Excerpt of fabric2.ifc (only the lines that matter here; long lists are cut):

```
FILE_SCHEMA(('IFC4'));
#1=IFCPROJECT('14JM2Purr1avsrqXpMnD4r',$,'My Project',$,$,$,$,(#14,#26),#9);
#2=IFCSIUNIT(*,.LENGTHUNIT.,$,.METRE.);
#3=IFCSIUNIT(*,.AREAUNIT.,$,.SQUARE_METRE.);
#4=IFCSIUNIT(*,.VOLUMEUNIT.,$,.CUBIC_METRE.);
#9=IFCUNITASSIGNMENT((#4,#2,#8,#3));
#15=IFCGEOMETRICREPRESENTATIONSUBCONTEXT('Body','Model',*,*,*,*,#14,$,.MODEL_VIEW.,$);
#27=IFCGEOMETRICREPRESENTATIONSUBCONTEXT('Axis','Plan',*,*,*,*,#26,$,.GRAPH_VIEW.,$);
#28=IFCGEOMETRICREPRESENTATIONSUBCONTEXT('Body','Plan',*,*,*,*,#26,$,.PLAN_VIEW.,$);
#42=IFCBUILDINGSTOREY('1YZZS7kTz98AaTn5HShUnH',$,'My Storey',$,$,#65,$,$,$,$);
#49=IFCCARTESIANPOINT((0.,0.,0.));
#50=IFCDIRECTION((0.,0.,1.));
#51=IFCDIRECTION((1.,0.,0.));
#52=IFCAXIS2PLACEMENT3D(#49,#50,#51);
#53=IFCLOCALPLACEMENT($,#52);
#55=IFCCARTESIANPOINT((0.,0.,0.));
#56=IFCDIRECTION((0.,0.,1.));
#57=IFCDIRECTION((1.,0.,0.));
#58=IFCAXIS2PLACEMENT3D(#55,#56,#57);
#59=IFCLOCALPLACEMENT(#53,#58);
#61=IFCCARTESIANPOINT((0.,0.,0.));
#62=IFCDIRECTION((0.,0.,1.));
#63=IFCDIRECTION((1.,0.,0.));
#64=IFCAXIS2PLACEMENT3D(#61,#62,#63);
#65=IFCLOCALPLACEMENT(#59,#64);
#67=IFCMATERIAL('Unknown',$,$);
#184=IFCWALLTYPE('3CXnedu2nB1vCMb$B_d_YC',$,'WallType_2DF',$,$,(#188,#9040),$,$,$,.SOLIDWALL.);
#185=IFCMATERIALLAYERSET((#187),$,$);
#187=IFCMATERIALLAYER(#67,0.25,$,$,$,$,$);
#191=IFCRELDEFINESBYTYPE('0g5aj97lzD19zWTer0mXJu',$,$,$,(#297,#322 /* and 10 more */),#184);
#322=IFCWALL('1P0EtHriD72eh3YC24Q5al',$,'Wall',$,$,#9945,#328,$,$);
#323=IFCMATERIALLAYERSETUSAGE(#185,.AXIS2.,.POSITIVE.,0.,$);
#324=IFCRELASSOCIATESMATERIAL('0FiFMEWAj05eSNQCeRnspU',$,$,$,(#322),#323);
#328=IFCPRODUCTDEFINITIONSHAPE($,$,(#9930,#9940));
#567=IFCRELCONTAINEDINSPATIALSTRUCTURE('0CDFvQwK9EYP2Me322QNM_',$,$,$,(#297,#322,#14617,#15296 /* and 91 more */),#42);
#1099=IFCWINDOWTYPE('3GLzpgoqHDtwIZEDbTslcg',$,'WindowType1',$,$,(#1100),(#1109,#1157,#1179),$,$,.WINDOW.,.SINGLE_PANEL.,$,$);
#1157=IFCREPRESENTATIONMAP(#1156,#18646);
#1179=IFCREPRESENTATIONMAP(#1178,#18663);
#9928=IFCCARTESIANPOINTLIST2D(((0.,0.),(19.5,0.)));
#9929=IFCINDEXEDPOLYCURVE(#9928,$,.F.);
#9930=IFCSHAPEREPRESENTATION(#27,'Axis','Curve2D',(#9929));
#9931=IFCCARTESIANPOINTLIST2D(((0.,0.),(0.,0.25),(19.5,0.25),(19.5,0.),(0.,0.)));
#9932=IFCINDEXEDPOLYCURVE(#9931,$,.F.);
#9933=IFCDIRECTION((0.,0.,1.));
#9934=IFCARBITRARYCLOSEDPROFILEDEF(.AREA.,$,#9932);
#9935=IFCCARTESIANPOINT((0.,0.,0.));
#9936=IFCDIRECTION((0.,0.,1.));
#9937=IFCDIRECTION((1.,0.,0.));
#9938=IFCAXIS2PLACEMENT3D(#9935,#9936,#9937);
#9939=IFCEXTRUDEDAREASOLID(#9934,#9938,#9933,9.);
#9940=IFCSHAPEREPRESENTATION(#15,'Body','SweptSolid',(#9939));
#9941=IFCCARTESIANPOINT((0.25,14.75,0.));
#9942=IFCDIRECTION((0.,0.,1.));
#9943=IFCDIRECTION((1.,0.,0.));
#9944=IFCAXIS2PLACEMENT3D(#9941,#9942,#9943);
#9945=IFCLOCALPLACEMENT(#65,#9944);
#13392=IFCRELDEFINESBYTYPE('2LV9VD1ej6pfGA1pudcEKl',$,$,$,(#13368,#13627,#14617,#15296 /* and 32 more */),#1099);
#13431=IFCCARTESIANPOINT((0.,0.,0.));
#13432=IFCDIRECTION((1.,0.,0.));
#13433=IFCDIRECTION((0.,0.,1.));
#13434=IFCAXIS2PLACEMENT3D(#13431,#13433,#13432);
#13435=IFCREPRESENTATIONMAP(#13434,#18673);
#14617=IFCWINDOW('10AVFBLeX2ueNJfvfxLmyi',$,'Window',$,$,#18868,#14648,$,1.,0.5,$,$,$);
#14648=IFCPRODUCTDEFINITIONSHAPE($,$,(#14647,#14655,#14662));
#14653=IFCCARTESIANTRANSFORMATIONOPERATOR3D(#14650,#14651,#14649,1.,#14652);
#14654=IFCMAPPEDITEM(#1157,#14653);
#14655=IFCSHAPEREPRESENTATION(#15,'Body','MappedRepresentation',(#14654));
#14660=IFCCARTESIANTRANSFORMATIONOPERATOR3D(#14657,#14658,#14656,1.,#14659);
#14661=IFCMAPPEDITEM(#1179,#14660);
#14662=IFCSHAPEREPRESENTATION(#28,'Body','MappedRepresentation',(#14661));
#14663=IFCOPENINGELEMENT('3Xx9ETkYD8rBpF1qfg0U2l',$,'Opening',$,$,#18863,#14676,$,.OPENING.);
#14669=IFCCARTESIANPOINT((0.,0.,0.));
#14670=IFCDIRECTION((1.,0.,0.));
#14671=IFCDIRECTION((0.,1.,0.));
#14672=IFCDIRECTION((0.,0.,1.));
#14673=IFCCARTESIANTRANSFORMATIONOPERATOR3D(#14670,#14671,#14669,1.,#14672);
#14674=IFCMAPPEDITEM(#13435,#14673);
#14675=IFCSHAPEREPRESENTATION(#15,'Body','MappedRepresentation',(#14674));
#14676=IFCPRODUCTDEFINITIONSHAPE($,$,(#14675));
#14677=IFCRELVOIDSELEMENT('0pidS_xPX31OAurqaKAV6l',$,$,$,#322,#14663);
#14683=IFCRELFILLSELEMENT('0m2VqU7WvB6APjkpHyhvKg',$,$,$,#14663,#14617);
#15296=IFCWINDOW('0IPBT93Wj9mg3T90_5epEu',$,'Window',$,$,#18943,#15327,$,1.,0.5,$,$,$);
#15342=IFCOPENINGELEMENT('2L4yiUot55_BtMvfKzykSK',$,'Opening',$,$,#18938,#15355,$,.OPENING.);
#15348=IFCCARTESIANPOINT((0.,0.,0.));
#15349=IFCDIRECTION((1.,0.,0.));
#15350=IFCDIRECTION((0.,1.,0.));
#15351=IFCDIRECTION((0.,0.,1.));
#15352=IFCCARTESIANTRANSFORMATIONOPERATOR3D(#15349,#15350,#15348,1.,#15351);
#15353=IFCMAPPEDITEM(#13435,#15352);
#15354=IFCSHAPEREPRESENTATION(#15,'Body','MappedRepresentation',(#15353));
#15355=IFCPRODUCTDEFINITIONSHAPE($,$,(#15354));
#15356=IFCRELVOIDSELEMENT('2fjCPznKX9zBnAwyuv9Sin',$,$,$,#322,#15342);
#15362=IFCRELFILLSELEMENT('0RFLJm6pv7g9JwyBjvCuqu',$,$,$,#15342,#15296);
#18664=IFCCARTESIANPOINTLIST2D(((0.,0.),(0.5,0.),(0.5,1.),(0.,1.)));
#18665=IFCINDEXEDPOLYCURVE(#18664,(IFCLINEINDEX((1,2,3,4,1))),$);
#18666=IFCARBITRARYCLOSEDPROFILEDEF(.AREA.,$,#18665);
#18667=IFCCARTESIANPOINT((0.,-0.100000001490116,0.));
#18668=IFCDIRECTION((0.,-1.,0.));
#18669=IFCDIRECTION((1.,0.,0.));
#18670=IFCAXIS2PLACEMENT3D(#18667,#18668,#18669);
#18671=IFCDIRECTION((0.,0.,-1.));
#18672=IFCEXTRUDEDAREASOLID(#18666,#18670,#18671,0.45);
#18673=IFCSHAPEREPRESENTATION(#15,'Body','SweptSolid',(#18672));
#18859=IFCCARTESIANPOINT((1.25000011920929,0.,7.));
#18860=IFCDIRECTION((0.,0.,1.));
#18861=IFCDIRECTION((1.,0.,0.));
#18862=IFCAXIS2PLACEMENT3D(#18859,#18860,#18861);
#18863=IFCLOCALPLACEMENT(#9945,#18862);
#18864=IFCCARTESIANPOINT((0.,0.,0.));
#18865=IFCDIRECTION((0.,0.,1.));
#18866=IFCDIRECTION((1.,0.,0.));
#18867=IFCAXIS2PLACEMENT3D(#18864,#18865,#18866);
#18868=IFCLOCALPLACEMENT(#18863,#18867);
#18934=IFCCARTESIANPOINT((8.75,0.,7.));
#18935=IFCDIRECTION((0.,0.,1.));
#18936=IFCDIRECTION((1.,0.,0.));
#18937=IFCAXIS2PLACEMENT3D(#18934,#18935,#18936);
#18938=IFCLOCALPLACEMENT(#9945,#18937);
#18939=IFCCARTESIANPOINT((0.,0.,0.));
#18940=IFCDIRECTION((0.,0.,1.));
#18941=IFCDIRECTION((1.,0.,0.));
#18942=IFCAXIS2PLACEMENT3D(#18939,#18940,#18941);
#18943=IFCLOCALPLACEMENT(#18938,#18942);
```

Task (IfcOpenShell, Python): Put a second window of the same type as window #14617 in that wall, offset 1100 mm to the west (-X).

```python
import ifcopenshell
import ifcopenshell.api.feature
import ifcopenshell.api.geometry
import ifcopenshell.api.root
import ifcopenshell.geom
import ifcopenshell.util.element
import ifcopenshell.util.placement
import ifcopenshell.util.shape
import ifcopenshell.util.unit

model = ifcopenshell.open("fabric2.ifc")
unit_scale = ifcopenshell.util.unit.calculate_unit_scale(model)
settings = ifcopenshell.geom.settings()


def volume(element):
    """Net volume in cubic metres, openings subtracted."""
    shape = ifcopenshell.geom.create_shape(settings, element)
    return ifcopenshell.util.shape.get_volume(shape.geometry)


window = model.by_guid("10AVFBLeX2ueNJfvfxLmyi")
opening = window.FillsVoids[0].RelatingOpeningElement
wall = opening.VoidsElements[0].RelatingBuildingElement
before = volume(wall)
shift = ifcopenshell.util.placement.get_local_placement(wall.ObjectPlacement)[:3, 0] * -1.1 / unit_scale

# copy_class copies the void relationship, type, container and properties, but no geometry.
new_opening = ifcopenshell.api.root.copy_class(model, product=opening)
new_opening.Representation = ifcopenshell.util.element.copy_deep(
    model, opening.Representation, exclude=["IfcGeometricRepresentationContext", "IfcRepresentationMap"]
)
new_window = ifcopenshell.api.root.copy_class(model, product=window)
new_window.Representation = ifcopenshell.util.element.copy_deep(
    model, window.Representation, exclude=["IfcGeometricRepresentationContext", "IfcRepresentationMap"]
)
ifcopenshell.api.feature.add_filling(model, opening=new_opening, element=new_window)

for old, new in ((opening, new_opening), (window, new_window)):
    matrix = ifcopenshell.util.placement.get_local_placement(old.ObjectPlacement)
    matrix[:3, 3] += shift
    ifcopenshell.api.geometry.edit_object_placement(model, product=new, matrix=matrix, is_si=False)

after = volume(wall)

print(f"wall volume {before:.3f} -> {after:.3f} m3")

model.write("fabric2_v2.ifc")
```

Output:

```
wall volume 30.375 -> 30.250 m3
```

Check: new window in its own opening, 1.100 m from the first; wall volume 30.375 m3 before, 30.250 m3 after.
